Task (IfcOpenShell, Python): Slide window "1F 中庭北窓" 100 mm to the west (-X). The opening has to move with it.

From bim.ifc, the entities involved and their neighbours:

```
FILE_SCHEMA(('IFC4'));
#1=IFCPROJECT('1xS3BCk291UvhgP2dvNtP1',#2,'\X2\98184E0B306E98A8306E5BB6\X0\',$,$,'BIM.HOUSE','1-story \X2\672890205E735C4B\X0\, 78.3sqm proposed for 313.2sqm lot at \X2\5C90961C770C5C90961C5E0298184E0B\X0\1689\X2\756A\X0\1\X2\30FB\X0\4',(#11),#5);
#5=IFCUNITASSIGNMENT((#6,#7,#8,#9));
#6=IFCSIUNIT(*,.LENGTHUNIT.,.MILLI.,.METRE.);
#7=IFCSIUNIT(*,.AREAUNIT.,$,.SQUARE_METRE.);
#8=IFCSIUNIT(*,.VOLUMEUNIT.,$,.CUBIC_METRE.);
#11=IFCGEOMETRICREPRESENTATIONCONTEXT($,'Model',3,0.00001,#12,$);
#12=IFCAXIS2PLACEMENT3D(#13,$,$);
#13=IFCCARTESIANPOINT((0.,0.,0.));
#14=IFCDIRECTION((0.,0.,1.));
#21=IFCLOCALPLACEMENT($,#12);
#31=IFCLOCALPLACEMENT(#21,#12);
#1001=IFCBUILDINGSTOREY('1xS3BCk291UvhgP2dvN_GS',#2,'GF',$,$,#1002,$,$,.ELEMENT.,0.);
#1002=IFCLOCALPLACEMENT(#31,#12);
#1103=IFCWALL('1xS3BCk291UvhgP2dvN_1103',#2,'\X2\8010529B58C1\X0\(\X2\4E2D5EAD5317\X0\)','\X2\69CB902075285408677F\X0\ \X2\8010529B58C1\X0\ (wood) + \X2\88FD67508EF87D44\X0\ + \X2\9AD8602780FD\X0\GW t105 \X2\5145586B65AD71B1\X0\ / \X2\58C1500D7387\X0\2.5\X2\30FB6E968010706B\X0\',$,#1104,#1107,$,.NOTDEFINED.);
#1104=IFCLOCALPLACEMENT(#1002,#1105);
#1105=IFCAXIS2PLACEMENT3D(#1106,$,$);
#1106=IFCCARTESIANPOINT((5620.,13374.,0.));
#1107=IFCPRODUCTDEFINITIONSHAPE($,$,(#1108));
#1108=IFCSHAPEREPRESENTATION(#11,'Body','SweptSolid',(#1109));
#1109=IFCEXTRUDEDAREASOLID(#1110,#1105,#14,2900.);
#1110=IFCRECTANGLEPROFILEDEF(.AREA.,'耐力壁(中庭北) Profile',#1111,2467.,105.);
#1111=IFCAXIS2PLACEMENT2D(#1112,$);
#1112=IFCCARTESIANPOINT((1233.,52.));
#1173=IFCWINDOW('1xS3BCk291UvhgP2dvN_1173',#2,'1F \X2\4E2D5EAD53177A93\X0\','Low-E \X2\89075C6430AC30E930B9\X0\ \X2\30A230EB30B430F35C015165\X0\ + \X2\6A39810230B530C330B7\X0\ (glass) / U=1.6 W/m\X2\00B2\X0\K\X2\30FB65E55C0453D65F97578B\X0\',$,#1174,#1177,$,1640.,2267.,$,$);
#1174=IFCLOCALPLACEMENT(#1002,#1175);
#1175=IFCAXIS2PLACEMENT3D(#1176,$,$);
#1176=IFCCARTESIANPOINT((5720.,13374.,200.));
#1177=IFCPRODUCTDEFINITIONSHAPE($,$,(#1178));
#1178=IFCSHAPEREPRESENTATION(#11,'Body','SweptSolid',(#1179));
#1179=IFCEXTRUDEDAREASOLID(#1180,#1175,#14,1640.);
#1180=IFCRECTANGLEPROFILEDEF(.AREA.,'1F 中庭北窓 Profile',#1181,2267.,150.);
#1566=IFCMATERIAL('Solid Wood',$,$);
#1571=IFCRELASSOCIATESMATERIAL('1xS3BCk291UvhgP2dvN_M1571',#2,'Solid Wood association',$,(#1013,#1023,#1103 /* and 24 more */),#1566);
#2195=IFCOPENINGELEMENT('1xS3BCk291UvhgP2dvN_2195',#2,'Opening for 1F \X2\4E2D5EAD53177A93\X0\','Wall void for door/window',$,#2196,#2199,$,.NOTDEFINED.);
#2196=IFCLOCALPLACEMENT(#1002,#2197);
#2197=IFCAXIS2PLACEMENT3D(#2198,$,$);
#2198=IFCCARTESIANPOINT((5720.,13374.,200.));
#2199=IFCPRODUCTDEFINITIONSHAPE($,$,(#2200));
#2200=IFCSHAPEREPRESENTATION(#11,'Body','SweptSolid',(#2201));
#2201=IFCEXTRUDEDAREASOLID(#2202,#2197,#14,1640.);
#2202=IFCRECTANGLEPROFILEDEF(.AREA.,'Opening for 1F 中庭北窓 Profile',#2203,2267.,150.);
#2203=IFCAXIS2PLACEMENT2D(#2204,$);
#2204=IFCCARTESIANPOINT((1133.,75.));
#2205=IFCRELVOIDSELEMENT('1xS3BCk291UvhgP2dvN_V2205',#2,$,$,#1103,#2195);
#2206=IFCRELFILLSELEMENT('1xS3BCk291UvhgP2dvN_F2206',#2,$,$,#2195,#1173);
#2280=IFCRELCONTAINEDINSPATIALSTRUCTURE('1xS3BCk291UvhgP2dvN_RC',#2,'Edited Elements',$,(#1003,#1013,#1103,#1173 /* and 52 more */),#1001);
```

```python
import ifcopenshell
import ifcopenshell.api.geometry
import ifcopenshell.util.placement

model = ifcopenshell.open("bim.ifc")

window = model.by_guid("1xS3BCk291UvhgP2dvN_1173")
opening = window.FillsVoids[0].RelatingOpeningElement
wall = opening.VoidsElements[0].RelatingBuildingElement

wall_matrix = ifcopenshell.util.placement.get_local_placement(wall.ObjectPlacement)
shift = wall_matrix[:3, 0] * -100.0
before = ifcopenshell.util.placement.get_local_placement(window.ObjectPlacement)[:3, 3].copy()

# The window is not placed relative to its opening, so move both.
for product in (opening, window):
    matrix = ifcopenshell.util.placement.get_local_placement(product.ObjectPlacement)
    matrix[:3, 3] += shift
    ifcopenshell.api.geometry.edit_object_placement(model, product=product, matrix=matrix, is_si=False)

after = ifcopenshell.util.placement.get_local_placement(window.ObjectPlacement)[:3, 3]
print("window moved by", (after - before).round(3) + 0.0)

model.write("bim-out.ifc")
```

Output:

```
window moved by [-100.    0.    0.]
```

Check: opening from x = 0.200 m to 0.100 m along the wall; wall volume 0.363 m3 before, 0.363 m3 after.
